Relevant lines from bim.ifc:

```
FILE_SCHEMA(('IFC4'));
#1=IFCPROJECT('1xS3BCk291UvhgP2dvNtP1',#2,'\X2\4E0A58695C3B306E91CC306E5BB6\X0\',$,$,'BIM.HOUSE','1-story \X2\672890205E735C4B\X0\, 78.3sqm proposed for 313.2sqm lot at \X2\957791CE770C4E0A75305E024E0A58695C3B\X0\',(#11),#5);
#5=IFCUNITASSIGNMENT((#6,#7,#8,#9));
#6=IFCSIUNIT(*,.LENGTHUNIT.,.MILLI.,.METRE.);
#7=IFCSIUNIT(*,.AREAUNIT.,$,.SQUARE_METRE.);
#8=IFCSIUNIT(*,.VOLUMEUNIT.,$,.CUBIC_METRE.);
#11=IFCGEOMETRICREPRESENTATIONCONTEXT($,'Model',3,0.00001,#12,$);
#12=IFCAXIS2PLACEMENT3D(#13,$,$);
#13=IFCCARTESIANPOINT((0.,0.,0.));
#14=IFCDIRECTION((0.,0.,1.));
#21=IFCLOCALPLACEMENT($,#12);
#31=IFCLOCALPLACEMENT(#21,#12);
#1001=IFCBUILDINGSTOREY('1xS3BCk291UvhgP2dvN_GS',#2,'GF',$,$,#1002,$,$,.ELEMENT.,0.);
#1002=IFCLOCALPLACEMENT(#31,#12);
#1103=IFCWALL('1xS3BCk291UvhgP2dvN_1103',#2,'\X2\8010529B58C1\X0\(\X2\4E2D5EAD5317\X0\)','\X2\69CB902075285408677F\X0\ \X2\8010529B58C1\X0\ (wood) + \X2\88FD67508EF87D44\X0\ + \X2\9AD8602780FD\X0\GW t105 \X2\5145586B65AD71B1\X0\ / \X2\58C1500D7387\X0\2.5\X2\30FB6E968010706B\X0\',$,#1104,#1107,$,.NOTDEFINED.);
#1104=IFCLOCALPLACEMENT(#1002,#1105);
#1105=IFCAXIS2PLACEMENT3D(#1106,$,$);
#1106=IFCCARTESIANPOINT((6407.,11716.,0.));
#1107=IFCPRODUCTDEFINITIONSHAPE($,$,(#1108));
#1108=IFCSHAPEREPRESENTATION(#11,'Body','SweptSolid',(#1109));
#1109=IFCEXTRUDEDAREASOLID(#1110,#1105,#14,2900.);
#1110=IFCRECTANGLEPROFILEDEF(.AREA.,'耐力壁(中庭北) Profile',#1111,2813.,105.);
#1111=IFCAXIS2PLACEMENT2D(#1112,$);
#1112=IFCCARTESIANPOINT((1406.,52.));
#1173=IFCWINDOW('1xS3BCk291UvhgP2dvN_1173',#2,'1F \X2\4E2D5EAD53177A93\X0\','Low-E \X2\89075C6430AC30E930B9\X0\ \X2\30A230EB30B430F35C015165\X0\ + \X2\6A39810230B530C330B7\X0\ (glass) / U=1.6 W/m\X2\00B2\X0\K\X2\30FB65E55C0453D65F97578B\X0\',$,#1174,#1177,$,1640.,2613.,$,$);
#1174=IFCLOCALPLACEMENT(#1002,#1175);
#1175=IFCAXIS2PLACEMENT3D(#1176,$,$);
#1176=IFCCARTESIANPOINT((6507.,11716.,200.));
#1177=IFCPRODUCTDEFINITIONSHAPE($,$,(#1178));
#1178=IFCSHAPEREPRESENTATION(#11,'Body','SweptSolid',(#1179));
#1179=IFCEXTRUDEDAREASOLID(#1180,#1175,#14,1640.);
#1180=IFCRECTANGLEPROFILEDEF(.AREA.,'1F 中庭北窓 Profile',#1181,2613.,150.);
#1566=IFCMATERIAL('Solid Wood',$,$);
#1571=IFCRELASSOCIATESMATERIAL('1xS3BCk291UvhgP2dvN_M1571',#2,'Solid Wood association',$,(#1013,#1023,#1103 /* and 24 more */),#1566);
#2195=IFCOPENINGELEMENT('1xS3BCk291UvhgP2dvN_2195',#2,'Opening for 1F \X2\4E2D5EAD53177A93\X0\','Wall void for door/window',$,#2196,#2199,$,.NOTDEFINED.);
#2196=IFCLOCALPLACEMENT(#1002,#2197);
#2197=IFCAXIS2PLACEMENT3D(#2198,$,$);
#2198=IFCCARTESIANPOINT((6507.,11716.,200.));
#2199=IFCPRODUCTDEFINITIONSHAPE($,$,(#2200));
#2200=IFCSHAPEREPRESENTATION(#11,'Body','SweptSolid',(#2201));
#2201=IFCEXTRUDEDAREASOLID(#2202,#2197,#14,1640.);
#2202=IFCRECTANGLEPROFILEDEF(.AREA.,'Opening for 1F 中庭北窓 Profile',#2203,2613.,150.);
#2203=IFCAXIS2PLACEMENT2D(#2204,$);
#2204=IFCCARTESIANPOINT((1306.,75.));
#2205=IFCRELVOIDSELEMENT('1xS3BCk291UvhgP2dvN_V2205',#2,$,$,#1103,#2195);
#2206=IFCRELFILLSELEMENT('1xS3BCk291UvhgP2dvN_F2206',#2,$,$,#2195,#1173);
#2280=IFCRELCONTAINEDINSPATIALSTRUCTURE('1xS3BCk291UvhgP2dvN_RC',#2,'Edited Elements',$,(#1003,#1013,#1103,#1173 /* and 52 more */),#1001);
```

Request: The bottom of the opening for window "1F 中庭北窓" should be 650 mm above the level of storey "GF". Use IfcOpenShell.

```python
import numpy as np
import ifcopenshell
import ifcopenshell.api.geometry
import ifcopenshell.geom
import ifcopenshell.util.element
import ifcopenshell.util.placement
import ifcopenshell.util.shape
import ifcopenshell.util.unit

model = ifcopenshell.open("bim.ifc")
unit_scale = ifcopenshell.util.unit.calculate_unit_scale(model)

window = model.by_guid("1xS3BCk291UvhgP2dvN_1173")
opening = window.FillsVoids[0].RelatingOpeningElement
storey = ifcopenshell.util.element.get_container(window, ifc_class="IfcBuildingStorey")
level = ifcopenshell.util.placement.get_local_placement(storey.ObjectPlacement)[2, 3]

# The opening's origin need not be at the sill, so measure its lowest point.
shape = ifcopenshell.geom.create_shape(ifcopenshell.geom.settings(), opening)
bottom = ifcopenshell.util.shape.get_shape_bottom_elevation(shape, shape.geometry) / unit_scale
dz = level + 0.65 / unit_scale - bottom

shift = np.array([0.0, 0.0, dz])
# The window is not placed relative to its opening, so move both.
for product in (opening, window):
    matrix = ifcopenshell.util.placement.get_local_placement(product.ObjectPlacement)
    matrix[:3, 3] += shift
    ifcopenshell.api.geometry.edit_object_placement(model, product=product, matrix=matrix, is_si=False)

print(f"moved by {dz * unit_scale:+.3f} m")

model.write("bim-out.ifc")
```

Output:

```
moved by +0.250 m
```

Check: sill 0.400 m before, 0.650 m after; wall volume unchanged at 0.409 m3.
